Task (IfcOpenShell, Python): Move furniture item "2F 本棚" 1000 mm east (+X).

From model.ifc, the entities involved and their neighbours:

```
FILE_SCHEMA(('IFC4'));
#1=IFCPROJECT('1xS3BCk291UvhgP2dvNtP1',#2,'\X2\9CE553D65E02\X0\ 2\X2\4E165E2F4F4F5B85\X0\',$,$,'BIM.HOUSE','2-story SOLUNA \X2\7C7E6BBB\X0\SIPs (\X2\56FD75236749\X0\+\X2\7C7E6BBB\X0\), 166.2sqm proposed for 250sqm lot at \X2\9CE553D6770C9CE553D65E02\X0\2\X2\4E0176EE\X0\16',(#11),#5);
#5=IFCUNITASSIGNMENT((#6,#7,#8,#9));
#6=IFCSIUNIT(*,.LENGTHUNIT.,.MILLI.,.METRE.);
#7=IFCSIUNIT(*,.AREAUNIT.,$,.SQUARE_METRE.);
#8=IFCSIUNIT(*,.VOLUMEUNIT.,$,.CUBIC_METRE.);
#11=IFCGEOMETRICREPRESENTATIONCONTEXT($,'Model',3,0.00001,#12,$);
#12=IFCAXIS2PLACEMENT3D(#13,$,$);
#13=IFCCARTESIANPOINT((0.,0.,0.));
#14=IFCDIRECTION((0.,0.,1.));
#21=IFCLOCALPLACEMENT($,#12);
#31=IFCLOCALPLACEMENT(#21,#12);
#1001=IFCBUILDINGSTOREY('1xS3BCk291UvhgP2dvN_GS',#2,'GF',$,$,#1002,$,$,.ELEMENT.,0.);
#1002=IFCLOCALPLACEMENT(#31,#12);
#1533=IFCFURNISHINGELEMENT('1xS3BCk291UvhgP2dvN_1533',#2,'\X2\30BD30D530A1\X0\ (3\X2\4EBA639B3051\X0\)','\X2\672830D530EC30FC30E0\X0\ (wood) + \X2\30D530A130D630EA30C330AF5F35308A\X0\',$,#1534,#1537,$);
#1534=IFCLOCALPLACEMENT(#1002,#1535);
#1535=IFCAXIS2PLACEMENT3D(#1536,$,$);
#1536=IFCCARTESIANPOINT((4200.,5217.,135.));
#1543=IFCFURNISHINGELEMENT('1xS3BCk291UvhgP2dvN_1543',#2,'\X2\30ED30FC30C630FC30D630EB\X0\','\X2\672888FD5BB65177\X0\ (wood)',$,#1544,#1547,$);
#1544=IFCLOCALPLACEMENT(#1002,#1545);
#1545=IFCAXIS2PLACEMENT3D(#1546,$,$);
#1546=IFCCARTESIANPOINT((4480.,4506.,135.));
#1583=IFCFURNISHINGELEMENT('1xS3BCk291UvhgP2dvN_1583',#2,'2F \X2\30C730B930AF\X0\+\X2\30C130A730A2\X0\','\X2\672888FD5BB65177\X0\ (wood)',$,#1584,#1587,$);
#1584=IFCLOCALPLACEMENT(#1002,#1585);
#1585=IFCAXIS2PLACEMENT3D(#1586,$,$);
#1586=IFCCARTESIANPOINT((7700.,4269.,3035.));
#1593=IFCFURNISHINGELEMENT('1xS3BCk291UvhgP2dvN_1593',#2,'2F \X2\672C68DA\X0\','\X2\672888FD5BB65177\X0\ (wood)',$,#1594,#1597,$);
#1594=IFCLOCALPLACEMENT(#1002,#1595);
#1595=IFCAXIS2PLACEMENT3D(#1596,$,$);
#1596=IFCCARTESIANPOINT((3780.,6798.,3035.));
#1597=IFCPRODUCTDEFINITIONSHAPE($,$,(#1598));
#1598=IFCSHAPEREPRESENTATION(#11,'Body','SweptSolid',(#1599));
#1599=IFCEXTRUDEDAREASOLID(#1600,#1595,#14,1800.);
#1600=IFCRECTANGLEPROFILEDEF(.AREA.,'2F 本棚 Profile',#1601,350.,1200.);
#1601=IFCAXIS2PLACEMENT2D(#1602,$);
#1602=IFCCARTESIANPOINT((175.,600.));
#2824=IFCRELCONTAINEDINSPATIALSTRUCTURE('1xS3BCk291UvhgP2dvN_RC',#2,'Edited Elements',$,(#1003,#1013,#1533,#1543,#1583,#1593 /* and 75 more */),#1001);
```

```python
import ifcopenshell
import ifcopenshell.api.geometry
import ifcopenshell.util.placement
import ifcopenshell.util.unit

model = ifcopenshell.open("model.ifc")
unit_scale = ifcopenshell.util.unit.calculate_unit_scale(model)

item = model.by_guid("1xS3BCk291UvhgP2dvN_1593")
matrix = ifcopenshell.util.placement.get_local_placement(item.ObjectPlacement)
matrix[0, 3] += 1 / unit_scale
ifcopenshell.api.geometry.edit_object_placement(model, product=item, matrix=matrix, is_si=False)

print(ifcopenshell.util.placement.get_local_placement(item.ObjectPlacement).round(3) + 0.0)

model.write("model-out.ifc")
```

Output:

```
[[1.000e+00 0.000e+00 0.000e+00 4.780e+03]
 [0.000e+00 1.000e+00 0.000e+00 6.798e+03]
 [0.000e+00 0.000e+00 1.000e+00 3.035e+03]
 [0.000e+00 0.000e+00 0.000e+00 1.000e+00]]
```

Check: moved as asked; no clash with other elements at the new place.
